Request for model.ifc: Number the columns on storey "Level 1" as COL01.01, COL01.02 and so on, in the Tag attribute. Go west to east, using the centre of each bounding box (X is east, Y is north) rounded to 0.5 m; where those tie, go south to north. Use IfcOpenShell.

First a look at what the model holds.

```python
import ifcopenshell
import ifcopenshell.util.element
import ifcopenshell.util.placement

model = ifcopenshell.open("model.ifc")
print(model.schema)
storey = next(s for s in model.by_type("IfcBuildingStorey") if s.Name == "Level 1")
columns = [e for e in ifcopenshell.util.element.get_decomposition(storey) if e.is_a("IfcColumn")]
for e in sorted(columns, key=lambda e: e.id()):
    origin = ifcopenshell.util.placement.get_local_placement(e.ObjectPlacement)[:3, 3]
    print(e.id(), e.Tag, e.Name, origin.round(2) + 0.0, sep=" | ")
```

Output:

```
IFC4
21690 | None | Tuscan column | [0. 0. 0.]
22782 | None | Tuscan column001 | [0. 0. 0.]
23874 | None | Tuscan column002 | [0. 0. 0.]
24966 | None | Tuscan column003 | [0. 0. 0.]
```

```python
import ifcopenshell
import ifcopenshell.geom
import ifcopenshell.util.element
import ifcopenshell.util.shape

model = ifcopenshell.open("model.ifc")
settings = ifcopenshell.geom.settings()
settings.set("use-world-coords", True)


def centre(element):
    shape = ifcopenshell.geom.create_shape(settings, element)
    return ifcopenshell.util.shape.get_bbox_centroid(shape.geometry)


storey = next(s for s in model.by_type("IfcBuildingStorey") if s.Name == "Level 1")
columns = [e for e in ifcopenshell.util.element.get_decomposition(storey) if e.is_a("IfcColumn")]

# Insertion points can sit at a corner or the storey origin, so sort by the geometry (in metres).
centres = {e: centre(e) for e in columns}
columns.sort(key=lambda e: (round(centres[e][0] / 0.5), centres[e][1]))

for i, e in enumerate(columns, start=1):
    number = f"COL01.{i:02d}"
    e.Tag = number
    print(e.id(), number)

model.write("model_v2.ifc")
```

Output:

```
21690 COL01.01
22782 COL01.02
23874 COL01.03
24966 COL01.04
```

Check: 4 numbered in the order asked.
